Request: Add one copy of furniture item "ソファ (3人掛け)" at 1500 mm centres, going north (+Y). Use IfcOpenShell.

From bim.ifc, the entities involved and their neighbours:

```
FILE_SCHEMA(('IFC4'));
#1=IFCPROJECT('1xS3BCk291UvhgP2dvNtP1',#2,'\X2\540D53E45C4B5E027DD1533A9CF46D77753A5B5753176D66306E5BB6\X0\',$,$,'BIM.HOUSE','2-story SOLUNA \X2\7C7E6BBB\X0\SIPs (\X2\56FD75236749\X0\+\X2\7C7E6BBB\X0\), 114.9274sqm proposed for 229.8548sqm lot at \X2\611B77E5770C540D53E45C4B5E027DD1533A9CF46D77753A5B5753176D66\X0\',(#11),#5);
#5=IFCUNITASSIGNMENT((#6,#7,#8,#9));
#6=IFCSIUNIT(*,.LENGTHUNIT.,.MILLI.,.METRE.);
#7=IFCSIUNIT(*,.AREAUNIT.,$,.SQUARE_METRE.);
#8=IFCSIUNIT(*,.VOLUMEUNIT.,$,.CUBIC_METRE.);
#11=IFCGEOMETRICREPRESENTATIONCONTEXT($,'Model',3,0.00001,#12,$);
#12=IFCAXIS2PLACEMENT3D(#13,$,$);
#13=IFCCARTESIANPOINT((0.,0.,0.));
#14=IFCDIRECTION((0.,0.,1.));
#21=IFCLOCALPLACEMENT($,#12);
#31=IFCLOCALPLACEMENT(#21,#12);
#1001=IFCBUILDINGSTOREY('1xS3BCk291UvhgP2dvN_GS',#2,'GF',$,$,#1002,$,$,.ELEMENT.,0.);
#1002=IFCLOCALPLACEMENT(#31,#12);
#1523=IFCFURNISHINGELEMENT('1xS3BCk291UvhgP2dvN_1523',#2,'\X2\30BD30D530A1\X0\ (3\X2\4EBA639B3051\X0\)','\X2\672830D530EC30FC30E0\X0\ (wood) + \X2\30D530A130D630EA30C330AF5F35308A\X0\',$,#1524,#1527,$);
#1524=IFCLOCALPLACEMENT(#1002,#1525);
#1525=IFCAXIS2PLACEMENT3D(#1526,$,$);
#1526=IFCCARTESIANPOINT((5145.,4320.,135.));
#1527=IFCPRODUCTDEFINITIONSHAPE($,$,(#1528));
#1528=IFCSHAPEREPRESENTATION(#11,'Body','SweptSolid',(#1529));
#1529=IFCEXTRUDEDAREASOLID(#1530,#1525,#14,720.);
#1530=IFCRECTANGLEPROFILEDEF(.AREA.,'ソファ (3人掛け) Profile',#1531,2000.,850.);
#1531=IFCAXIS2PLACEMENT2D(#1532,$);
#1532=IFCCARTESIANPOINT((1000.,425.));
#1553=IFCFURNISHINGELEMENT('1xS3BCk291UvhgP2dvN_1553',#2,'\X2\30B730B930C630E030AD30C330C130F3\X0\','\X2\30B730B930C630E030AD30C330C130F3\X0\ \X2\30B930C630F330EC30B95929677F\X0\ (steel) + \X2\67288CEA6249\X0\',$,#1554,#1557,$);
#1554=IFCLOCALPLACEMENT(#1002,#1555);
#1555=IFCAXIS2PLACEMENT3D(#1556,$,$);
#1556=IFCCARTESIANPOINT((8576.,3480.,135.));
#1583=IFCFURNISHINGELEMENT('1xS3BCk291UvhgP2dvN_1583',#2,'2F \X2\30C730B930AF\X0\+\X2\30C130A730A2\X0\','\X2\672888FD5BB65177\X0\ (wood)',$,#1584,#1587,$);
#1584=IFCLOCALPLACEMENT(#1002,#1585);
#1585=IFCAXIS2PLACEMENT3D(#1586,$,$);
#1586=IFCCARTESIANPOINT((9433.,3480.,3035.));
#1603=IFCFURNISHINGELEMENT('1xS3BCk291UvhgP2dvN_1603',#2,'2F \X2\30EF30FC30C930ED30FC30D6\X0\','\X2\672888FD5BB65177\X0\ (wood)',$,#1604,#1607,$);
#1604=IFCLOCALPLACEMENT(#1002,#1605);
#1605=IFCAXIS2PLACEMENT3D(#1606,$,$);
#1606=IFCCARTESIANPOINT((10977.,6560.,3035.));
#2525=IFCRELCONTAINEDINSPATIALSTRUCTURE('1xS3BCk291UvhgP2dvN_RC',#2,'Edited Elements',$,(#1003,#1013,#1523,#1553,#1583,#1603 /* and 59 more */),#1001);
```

```python
import numpy as np
import ifcopenshell
import ifcopenshell.api.geometry
import ifcopenshell.api.root
import ifcopenshell.util.element
import ifcopenshell.util.placement
import ifcopenshell.util.unit

model = ifcopenshell.open("bim.ifc")
unit_scale = ifcopenshell.util.unit.calculate_unit_scale(model)


def reuse_history(source, copy):
    """copy_class also copies each property set's owner history, people and application; keep the originals."""
    for rel in copy.IsDefinedBy:
        if rel.is_a("IfcRelDefinesByProperties") and (history := rel.RelatingPropertyDefinition.OwnerHistory):
            rel.RelatingPropertyDefinition.OwnerHistory = source.OwnerHistory
            ifcopenshell.util.element.remove_deep2(model, history)


source = model.by_guid("1xS3BCk291UvhgP2dvN_1523")
base = ifcopenshell.util.placement.get_local_placement(source.ObjectPlacement)
step = np.array([0.0, 1.0, 0.0]) * 1.5 / unit_scale

for i in range(1, 2):
    copy = ifcopenshell.api.root.copy_class(model, product=source)
    copy.Representation = ifcopenshell.util.element.copy_deep(
        model, source.Representation, exclude=["IfcGeometricRepresentationContext", "IfcRepresentationMap"]
    )
    reuse_history(source, copy)
    matrix = base.copy()
    matrix[:3, 3] += i * step
    print("added at", matrix[:3, 3].round(3) + 0.0)
    ifcopenshell.api.geometry.edit_object_placement(model, product=copy, matrix=matrix, is_si=False)

model.write("bim_rev.ifc")
```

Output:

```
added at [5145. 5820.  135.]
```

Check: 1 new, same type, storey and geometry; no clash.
